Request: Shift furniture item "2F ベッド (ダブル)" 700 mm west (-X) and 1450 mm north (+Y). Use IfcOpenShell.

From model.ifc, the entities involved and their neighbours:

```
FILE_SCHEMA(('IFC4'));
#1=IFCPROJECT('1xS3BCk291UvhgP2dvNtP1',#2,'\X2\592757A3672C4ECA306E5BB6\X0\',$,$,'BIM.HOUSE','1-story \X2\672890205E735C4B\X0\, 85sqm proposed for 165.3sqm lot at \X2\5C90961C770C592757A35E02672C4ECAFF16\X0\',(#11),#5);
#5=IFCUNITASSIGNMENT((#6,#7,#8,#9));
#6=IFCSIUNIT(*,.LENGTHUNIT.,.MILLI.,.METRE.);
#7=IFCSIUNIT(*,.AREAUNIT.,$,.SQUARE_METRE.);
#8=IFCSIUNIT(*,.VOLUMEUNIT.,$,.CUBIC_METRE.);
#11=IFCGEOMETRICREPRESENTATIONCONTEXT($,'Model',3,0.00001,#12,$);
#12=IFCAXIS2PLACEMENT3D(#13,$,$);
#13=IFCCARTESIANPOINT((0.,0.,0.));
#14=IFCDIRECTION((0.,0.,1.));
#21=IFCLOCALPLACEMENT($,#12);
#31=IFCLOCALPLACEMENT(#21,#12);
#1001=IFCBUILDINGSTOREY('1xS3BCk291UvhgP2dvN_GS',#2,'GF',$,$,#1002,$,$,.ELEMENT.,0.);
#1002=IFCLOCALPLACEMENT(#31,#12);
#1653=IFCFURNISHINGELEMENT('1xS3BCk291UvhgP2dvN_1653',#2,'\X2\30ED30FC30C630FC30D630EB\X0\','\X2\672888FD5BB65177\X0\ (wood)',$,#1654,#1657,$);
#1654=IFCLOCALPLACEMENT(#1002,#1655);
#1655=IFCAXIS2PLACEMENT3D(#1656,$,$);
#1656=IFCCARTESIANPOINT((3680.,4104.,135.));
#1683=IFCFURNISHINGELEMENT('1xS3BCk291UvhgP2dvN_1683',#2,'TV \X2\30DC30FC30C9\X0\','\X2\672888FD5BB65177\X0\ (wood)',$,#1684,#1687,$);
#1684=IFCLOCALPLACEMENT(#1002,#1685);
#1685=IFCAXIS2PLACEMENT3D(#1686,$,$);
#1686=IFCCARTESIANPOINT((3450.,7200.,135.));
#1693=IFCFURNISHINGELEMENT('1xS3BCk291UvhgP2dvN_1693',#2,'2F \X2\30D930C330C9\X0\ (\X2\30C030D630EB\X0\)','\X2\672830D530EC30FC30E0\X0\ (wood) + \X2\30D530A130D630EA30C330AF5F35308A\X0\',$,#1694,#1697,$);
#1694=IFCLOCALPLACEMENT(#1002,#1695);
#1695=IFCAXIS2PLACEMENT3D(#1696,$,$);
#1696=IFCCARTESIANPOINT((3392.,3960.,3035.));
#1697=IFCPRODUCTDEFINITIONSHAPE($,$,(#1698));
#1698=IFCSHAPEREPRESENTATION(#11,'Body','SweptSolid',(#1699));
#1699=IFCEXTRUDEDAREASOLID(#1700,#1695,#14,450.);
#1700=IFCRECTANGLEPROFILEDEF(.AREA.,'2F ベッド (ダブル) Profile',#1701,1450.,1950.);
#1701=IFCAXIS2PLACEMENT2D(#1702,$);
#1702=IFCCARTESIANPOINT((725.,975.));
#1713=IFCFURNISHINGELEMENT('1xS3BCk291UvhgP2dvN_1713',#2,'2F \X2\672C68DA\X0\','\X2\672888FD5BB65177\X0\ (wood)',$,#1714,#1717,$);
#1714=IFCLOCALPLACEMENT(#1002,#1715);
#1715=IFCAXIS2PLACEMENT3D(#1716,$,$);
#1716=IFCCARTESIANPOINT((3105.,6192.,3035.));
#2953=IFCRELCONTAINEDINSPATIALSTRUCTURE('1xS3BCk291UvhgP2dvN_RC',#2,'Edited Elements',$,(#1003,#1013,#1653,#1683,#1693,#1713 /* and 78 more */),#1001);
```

```python
import ifcopenshell
import ifcopenshell.api.geometry
import ifcopenshell.util.placement
import ifcopenshell.util.unit

model = ifcopenshell.open("model.ifc")
unit_scale = ifcopenshell.util.unit.calculate_unit_scale(model)

item = model.by_guid("1xS3BCk291UvhgP2dvN_1693")
matrix = ifcopenshell.util.placement.get_local_placement(item.ObjectPlacement)
matrix[0, 3] -= 0.7 / unit_scale
matrix[1, 3] += 1.45 / unit_scale
ifcopenshell.api.geometry.edit_object_placement(model, product=item, matrix=matrix, is_si=False)

print(ifcopenshell.util.placement.get_local_placement(item.ObjectPlacement).round(3) + 0.0)

model.write("model_updated.ifc")
```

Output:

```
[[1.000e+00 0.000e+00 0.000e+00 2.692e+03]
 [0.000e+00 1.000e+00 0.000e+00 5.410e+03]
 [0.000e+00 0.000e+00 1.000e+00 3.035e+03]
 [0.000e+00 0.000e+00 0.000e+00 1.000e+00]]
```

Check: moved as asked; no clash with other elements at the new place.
